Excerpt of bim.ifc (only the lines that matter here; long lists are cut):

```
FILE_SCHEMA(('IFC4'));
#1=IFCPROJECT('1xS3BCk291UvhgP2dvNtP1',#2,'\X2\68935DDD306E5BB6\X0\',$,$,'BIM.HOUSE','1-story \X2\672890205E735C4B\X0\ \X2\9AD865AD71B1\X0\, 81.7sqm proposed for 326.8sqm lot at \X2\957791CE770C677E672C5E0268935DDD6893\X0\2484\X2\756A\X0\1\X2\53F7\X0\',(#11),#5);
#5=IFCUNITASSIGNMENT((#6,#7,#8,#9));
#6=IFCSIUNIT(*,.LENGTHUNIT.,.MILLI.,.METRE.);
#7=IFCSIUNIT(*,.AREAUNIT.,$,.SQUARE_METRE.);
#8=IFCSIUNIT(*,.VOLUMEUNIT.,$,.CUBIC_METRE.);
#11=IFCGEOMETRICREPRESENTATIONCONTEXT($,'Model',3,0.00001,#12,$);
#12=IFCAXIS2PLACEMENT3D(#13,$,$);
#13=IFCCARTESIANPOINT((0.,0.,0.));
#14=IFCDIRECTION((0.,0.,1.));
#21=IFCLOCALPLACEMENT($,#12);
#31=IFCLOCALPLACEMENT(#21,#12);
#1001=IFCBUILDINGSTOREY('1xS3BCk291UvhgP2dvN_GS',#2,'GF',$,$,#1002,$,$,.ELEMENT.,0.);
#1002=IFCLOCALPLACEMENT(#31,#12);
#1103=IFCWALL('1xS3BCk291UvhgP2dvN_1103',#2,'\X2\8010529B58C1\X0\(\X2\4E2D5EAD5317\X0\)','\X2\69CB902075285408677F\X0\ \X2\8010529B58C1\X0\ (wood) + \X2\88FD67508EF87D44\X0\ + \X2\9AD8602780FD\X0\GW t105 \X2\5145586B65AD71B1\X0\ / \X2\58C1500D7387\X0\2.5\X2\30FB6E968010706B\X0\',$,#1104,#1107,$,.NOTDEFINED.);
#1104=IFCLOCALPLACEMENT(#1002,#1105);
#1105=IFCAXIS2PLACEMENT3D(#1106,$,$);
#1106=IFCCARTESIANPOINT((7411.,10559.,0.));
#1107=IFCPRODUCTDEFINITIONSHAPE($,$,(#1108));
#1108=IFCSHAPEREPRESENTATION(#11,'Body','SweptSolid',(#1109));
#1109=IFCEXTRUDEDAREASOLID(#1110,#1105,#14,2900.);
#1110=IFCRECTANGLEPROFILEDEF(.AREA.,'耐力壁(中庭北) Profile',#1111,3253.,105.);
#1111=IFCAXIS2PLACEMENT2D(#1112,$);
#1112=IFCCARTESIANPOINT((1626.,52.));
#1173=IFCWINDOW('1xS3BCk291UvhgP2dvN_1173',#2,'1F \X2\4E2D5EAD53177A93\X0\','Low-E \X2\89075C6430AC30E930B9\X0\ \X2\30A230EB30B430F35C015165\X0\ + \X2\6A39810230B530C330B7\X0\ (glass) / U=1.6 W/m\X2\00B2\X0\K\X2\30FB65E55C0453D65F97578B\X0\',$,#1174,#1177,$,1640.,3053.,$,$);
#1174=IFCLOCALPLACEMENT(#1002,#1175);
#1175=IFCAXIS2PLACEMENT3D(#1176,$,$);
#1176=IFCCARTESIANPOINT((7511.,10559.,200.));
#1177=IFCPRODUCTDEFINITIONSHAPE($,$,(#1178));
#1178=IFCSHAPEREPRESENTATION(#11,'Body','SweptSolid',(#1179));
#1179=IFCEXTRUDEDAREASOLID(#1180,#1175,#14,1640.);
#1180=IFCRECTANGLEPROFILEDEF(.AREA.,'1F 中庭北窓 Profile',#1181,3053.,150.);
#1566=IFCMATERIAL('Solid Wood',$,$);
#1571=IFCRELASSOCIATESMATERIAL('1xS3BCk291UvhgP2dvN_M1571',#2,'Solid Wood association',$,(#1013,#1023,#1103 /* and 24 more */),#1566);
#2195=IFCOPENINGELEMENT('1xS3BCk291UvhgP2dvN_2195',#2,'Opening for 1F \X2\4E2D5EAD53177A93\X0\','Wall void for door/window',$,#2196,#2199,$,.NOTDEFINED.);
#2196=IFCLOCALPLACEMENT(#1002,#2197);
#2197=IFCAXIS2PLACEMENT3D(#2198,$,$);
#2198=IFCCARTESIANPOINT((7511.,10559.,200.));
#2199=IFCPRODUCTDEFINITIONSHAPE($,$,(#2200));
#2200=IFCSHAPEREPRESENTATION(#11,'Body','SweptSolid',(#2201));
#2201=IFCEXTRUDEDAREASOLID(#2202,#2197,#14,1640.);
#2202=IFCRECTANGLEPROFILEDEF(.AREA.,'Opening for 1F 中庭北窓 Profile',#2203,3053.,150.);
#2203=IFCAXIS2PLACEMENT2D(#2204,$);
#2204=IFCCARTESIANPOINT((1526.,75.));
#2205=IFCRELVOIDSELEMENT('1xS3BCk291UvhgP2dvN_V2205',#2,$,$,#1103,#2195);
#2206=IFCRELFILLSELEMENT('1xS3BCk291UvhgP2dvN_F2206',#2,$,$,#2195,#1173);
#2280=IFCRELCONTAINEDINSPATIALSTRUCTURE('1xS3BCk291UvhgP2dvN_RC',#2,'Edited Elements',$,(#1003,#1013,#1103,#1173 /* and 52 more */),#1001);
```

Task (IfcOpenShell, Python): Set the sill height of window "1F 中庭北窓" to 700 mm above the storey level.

```python
import numpy as np
import ifcopenshell
import ifcopenshell.api.geometry
import ifcopenshell.geom
import ifcopenshell.util.element
import ifcopenshell.util.placement
import ifcopenshell.util.shape
import ifcopenshell.util.unit

model = ifcopenshell.open("bim.ifc")
unit_scale = ifcopenshell.util.unit.calculate_unit_scale(model)

window = model.by_guid("1xS3BCk291UvhgP2dvN_1173")
opening = window.FillsVoids[0].RelatingOpeningElement
storey = ifcopenshell.util.element.get_container(window, ifc_class="IfcBuildingStorey")
level = ifcopenshell.util.placement.get_local_placement(storey.ObjectPlacement)[2, 3]

# The opening's origin need not be at the sill, so measure its lowest point.
shape = ifcopenshell.geom.create_shape(ifcopenshell.geom.settings(), opening)
bottom = ifcopenshell.util.shape.get_shape_bottom_elevation(shape, shape.geometry) / unit_scale
dz = level + 0.7 / unit_scale - bottom

shift = np.array([0.0, 0.0, dz])
# The window is not placed relative to its opening, so move both.
for product in (opening, window):
    matrix = ifcopenshell.util.placement.get_local_placement(product.ObjectPlacement)
    matrix[:3, 3] += shift
    ifcopenshell.api.geometry.edit_object_placement(model, product=product, matrix=matrix, is_si=False)

print(f"moved by {dz * unit_scale:+.3f} m")

model.write("bim_v2.ifc")
```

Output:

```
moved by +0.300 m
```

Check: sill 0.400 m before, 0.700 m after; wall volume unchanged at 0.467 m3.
